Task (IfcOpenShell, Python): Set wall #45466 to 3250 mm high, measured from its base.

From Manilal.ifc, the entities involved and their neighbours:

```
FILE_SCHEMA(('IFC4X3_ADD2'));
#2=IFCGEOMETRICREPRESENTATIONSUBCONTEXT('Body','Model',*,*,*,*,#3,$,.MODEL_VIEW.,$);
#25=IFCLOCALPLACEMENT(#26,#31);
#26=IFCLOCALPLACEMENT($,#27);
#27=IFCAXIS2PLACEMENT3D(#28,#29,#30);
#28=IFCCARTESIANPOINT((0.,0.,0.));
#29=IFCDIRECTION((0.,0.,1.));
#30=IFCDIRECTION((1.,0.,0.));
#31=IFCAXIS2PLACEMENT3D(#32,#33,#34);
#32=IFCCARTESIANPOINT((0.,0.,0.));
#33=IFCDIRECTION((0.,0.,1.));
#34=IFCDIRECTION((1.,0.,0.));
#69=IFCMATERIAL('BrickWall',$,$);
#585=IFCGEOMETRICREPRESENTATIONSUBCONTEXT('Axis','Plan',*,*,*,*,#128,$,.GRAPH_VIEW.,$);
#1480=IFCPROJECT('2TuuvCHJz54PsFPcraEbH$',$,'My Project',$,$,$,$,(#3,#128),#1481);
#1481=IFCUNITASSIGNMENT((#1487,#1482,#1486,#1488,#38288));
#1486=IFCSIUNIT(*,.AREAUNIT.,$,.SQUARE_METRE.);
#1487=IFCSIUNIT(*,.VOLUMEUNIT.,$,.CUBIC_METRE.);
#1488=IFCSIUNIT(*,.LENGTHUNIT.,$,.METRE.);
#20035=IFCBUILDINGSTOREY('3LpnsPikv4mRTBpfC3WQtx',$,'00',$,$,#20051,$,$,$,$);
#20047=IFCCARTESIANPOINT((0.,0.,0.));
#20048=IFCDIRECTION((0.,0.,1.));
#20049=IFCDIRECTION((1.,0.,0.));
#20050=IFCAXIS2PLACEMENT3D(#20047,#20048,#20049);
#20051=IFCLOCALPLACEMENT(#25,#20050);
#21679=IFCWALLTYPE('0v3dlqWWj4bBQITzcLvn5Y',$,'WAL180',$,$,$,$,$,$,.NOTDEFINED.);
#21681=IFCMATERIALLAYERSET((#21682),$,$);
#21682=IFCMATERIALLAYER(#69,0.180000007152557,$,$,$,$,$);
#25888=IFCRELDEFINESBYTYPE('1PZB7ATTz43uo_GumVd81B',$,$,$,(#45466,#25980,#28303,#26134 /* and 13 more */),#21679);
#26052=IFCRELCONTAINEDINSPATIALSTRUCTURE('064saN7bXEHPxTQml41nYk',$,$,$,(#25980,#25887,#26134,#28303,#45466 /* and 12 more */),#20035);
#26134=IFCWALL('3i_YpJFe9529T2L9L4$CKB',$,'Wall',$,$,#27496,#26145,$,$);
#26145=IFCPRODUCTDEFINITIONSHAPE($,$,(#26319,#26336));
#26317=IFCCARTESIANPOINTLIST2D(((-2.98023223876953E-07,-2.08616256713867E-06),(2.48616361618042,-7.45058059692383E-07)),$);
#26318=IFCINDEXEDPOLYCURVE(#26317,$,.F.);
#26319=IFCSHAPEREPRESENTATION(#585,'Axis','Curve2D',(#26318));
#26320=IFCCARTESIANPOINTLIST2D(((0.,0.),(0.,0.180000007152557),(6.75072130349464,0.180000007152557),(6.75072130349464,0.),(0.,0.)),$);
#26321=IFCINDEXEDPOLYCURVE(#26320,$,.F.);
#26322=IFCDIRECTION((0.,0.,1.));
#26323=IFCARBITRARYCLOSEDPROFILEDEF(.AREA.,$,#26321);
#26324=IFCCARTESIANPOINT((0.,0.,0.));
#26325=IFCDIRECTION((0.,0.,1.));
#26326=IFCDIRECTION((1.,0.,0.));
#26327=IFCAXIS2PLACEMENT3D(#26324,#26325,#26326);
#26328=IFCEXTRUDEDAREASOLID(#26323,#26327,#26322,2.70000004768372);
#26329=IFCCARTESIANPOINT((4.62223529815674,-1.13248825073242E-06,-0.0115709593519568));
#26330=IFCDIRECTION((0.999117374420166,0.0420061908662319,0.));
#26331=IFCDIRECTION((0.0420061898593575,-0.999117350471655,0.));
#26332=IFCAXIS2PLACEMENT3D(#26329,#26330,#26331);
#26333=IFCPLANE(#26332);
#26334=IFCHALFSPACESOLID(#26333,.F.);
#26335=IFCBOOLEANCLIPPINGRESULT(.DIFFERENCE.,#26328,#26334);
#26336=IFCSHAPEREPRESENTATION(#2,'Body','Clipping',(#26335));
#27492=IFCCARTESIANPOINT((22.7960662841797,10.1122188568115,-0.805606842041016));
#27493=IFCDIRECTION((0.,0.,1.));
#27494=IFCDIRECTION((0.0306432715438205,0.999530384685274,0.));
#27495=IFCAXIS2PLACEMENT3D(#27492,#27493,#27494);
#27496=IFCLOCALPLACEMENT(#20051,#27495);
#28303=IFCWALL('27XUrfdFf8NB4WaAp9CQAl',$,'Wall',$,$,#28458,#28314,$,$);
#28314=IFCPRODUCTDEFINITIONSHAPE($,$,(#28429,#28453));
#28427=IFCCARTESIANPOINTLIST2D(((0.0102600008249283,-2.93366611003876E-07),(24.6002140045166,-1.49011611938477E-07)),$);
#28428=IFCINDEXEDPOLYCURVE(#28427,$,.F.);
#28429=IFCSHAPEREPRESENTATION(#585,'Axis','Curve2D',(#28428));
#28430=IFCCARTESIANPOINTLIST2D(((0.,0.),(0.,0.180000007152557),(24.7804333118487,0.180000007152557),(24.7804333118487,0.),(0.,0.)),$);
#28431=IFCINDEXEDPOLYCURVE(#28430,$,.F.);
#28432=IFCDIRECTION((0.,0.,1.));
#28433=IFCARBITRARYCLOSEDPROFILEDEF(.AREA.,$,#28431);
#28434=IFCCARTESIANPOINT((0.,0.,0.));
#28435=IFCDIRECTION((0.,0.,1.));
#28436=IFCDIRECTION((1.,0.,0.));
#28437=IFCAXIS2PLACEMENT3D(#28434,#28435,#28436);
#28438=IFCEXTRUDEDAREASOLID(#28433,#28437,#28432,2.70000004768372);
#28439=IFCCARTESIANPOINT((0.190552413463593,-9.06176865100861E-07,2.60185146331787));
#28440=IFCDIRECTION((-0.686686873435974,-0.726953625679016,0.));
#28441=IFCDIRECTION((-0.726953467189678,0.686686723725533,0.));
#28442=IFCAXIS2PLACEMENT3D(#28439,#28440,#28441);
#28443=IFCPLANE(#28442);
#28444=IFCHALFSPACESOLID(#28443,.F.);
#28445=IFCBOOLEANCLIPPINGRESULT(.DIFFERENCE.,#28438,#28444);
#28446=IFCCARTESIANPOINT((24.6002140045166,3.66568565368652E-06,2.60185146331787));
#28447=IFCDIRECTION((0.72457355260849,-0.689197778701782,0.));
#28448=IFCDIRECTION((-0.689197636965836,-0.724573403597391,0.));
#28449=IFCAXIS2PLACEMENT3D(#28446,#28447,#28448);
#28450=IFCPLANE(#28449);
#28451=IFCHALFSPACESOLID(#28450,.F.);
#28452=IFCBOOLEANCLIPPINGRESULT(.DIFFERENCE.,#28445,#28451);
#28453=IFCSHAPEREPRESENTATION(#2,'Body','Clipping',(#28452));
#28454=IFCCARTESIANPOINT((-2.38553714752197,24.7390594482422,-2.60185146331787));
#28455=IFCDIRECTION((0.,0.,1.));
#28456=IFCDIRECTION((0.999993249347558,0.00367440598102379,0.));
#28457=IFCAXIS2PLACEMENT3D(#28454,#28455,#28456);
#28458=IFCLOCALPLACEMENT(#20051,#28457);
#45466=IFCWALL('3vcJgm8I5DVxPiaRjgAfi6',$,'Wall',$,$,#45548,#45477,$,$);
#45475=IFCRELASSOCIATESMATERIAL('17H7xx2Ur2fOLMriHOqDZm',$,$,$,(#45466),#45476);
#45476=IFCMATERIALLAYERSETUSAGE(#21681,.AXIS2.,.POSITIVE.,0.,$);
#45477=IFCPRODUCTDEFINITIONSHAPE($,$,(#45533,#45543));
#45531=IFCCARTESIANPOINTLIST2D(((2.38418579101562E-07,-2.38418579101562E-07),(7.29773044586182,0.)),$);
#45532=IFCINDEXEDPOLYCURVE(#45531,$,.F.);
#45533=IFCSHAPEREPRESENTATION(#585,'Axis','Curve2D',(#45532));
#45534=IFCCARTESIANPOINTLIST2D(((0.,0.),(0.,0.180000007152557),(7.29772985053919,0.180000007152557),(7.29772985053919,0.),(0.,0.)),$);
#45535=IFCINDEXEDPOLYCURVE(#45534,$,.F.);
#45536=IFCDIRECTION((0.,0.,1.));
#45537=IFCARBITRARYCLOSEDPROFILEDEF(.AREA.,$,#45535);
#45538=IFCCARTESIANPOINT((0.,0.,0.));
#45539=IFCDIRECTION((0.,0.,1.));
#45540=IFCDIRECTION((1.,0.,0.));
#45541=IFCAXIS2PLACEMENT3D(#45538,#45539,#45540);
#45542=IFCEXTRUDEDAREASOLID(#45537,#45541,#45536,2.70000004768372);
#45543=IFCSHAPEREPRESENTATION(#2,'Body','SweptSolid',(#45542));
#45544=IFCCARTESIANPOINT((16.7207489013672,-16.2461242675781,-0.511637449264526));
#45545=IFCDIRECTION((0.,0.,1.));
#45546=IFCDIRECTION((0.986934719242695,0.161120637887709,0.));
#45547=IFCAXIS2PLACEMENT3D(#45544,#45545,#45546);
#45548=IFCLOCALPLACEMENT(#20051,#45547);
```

```python
import ifcopenshell
import ifcopenshell.geom
import ifcopenshell.util.representation
import ifcopenshell.util.shape
import ifcopenshell.util.unit

model = ifcopenshell.open("Manilal.ifc")
unit_scale = ifcopenshell.util.unit.calculate_unit_scale(model)
settings = ifcopenshell.geom.settings()


def volume(element):
    """Net volume in cubic metres, openings subtracted."""
    shape = ifcopenshell.geom.create_shape(settings, element)
    return ifcopenshell.util.shape.get_volume(shape.geometry)


wall = model.by_guid("3vcJgm8I5DVxPiaRjgAfi6")
before = volume(wall)

body = ifcopenshell.util.representation.get_representation(wall, "Model", "Body")
solid = body.Items[0]
old_height = solid.Depth
solid.Depth = 3.25 / unit_scale
after = volume(wall)

print(f"height {old_height:g} -> {solid.Depth:g}, volume {before:.3f} -> {after:.3f} m3")

model.write("Manilal_v2.ifc")
```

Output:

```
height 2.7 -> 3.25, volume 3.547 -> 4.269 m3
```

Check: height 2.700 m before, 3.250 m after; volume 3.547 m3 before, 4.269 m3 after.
